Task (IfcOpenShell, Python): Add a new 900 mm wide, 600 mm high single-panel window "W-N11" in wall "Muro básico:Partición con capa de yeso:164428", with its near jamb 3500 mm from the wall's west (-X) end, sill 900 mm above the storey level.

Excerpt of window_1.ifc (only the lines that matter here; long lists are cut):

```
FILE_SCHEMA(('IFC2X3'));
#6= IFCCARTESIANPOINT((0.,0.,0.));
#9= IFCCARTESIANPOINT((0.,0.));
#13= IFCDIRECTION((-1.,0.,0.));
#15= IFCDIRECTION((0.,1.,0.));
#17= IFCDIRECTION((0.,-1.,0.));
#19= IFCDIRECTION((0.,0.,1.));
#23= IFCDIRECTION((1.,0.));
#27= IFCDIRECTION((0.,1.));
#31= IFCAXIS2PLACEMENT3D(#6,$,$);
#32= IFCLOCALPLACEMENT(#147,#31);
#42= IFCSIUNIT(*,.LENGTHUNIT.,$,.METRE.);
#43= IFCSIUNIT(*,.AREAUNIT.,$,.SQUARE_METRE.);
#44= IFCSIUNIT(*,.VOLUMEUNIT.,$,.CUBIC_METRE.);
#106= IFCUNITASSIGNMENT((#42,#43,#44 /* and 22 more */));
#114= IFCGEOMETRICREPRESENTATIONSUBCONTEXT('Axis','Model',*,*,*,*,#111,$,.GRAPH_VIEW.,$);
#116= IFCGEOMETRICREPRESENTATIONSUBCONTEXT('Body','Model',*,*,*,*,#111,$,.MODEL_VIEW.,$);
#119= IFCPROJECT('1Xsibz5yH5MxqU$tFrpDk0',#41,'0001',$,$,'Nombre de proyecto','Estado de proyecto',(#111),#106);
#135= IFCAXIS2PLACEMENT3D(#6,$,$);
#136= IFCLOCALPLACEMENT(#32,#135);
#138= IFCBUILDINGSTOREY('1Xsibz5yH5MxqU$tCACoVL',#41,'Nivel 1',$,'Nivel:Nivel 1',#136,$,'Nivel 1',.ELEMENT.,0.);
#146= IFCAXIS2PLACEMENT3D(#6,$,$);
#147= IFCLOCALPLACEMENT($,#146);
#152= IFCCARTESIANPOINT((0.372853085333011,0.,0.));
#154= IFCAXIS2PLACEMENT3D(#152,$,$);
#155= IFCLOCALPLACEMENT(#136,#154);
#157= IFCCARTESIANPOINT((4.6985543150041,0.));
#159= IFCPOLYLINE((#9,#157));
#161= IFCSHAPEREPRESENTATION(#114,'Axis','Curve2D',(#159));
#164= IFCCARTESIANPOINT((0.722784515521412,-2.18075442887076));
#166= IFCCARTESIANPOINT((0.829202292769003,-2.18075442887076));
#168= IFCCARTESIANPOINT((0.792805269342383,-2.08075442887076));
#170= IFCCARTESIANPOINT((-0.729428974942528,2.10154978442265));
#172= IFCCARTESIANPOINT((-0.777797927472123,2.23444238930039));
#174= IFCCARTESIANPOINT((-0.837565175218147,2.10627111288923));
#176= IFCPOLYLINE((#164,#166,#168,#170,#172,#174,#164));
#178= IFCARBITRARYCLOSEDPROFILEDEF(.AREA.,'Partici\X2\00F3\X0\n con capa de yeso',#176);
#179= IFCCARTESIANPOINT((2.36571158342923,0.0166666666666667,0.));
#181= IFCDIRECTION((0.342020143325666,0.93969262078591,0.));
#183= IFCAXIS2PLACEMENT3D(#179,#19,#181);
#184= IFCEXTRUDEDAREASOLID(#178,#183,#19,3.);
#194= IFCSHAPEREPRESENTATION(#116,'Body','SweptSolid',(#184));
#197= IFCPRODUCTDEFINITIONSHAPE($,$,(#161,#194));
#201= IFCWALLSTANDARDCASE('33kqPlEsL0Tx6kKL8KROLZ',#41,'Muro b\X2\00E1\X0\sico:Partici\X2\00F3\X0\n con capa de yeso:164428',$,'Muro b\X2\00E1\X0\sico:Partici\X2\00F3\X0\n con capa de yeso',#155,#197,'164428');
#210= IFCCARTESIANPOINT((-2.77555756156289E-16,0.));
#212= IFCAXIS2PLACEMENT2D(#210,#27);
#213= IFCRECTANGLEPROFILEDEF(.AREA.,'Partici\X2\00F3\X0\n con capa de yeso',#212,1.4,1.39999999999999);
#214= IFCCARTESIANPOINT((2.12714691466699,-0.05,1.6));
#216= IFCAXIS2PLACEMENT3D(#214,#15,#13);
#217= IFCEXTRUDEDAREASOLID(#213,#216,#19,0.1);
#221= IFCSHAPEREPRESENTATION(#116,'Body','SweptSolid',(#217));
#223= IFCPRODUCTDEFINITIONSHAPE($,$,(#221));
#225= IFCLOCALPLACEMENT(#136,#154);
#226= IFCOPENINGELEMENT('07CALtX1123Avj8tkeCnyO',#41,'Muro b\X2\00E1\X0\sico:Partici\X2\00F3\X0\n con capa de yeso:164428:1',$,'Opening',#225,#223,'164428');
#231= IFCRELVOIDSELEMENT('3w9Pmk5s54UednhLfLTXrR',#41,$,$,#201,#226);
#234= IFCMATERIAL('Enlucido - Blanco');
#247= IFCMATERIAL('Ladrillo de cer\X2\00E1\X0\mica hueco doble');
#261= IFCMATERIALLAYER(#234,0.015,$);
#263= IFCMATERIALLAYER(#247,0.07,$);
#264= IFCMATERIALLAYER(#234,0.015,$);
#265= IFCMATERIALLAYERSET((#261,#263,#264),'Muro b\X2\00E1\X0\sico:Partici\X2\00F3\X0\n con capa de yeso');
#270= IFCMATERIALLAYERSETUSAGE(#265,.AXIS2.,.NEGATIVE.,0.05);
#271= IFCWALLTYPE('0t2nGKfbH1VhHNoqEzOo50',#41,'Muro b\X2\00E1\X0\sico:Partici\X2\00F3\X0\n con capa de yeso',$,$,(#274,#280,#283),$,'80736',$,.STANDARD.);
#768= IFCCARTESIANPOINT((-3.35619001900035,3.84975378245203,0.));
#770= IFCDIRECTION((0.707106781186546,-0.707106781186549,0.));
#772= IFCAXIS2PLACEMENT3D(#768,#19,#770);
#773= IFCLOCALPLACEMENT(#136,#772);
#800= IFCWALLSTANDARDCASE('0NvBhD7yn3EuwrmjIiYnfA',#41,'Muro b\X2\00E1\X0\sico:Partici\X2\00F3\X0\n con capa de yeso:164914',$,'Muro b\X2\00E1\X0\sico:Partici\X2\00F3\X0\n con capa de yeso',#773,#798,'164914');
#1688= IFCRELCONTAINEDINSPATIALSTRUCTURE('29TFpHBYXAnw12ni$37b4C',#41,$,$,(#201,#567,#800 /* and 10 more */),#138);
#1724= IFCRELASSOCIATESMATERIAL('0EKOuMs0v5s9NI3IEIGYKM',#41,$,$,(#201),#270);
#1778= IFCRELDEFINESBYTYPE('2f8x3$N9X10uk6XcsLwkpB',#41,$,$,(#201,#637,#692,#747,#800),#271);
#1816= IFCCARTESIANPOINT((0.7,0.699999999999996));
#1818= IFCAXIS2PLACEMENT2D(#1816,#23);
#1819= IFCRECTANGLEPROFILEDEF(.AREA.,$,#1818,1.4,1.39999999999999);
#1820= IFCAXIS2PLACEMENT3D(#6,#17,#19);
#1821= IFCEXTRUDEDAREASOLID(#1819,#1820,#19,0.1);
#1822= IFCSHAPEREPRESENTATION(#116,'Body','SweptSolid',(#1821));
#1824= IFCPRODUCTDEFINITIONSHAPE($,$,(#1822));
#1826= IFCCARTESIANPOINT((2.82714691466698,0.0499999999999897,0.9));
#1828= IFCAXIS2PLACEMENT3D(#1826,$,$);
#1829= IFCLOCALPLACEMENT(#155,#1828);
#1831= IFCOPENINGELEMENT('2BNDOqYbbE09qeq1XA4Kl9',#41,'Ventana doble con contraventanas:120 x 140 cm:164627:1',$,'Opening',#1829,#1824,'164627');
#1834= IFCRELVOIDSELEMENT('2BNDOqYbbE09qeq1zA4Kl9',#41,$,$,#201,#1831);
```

```python
import numpy as np
import ifcopenshell
import ifcopenshell.api.feature
import ifcopenshell.api.geometry
import ifcopenshell.api.root
import ifcopenshell.api.spatial
import ifcopenshell.api.type
import ifcopenshell.geom
import ifcopenshell.util.element
import ifcopenshell.util.placement
import ifcopenshell.util.representation
import ifcopenshell.util.shape
import ifcopenshell.util.unit

model = ifcopenshell.open("window_1.ifc")
unit_scale = ifcopenshell.util.unit.calculate_unit_scale(model)
settings = ifcopenshell.geom.settings()


def volume(element):
    """Net volume in cubic metres, openings subtracted."""
    shape = ifcopenshell.geom.create_shape(settings, element)
    return ifcopenshell.util.shape.get_volume(shape.geometry)


wall = model.by_guid("33kqPlEsL0Tx6kKL8KROLZ")
storey = ifcopenshell.util.element.get_container(wall, ifc_class="IfcBuildingStorey")
context = ifcopenshell.util.representation.get_context(model, "Model", "Body", "MODEL_VIEW")
before = volume(wall)

width, height, from_end, sill = 0.9, 0.6, 3.5, 0.9  # metres

# The wall runs along its own X axis, and the end named is its -X end.
wall_shape = ifcopenshell.geom.create_shape(settings, wall)
x, y, z = ifcopenshell.util.shape.get_vertices(wall_shape.geometry).T
start = x.min() + from_end
face, thickness = float(y.min()), float(y.max() - y.min())
wall_matrix = ifcopenshell.util.placement.get_local_placement(wall.ObjectPlacement)
level = ifcopenshell.util.placement.get_local_placement(storey.ObjectPlacement)[2, 3]


def in_wall(x, y):
    """Placement at x, y metres in the wall's axes, at sill height."""
    matrix = wall_matrix.copy()
    matrix[:, 3] = wall_matrix @ np.array([x / unit_scale, y / unit_scale, 0.0, 1.0])
    matrix[2, 3] = level + sill / unit_scale
    return matrix


# Opening: a box that overshoots both wall faces by 50 mm.
opening = ifcopenshell.api.root.create_entity(model, ifc_class="IfcOpeningElement")
box = ifcopenshell.api.geometry.add_wall_representation(
    model, context=context, length=width, height=height, thickness=thickness + 0.1
)
ifcopenshell.api.geometry.assign_representation(model, product=opening, representation=box)
ifcopenshell.api.geometry.edit_object_placement(model, product=opening, matrix=in_wall(start, face - 0.05), is_si=False)
ifcopenshell.api.feature.add_feature(model, feature=opening, element=wall)

window = ifcopenshell.api.root.create_entity(model, ifc_class="IfcWindow", name="W-N11")
window.OverallWidth, window.OverallHeight = width / unit_scale, height / unit_scale
body = ifcopenshell.api.geometry.add_window_representation(
    model,
    context=context,
    overall_width=window.OverallWidth,
    overall_height=window.OverallHeight,
    partition_type="SINGLE_PANEL",
)
ifcopenshell.api.geometry.assign_representation(model, product=window, representation=body)
ifcopenshell.api.spatial.assign_container(model, products=[window], relating_structure=storey)
fills = ifcopenshell.api.feature.add_filling(model, opening=opening, element=window)
fills.OwnerHistory = window.OwnerHistory  # required in IFC2X3

# IFC2X3 keeps the operation on the window style.
style = ifcopenshell.api.root.create_entity(model, ifc_class="IfcWindowStyle", name="W-N11")
style.OperationType, style.ConstructionType = "SINGLE_PANEL", "NOTDEFINED"
style.ParameterTakesPrecedence = style.Sizeable = False
ifcopenshell.api.type.assign_type(model, related_objects=[window], relating_type=style)

# Centre the window in the wall's thickness.
ifcopenshell.api.geometry.edit_object_placement(model, product=window, matrix=in_wall(start, face), is_si=False)
window_shape = ifcopenshell.geom.create_shape(settings, window)
depth = ifcopenshell.util.shape.get_vertices(window_shape.geometry)[:, 1]
offset = face + thickness / 2 - (depth.min() + depth.max()) / 2
ifcopenshell.api.geometry.edit_object_placement(model, product=window, matrix=in_wall(start, offset), is_si=False)

after = volume(wall)

print(f"wall volume {before:.3f} -> {after:.3f} m3")

model.write("window_1_v2.ifc")
```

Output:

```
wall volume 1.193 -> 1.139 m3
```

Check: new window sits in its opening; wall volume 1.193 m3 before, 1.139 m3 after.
